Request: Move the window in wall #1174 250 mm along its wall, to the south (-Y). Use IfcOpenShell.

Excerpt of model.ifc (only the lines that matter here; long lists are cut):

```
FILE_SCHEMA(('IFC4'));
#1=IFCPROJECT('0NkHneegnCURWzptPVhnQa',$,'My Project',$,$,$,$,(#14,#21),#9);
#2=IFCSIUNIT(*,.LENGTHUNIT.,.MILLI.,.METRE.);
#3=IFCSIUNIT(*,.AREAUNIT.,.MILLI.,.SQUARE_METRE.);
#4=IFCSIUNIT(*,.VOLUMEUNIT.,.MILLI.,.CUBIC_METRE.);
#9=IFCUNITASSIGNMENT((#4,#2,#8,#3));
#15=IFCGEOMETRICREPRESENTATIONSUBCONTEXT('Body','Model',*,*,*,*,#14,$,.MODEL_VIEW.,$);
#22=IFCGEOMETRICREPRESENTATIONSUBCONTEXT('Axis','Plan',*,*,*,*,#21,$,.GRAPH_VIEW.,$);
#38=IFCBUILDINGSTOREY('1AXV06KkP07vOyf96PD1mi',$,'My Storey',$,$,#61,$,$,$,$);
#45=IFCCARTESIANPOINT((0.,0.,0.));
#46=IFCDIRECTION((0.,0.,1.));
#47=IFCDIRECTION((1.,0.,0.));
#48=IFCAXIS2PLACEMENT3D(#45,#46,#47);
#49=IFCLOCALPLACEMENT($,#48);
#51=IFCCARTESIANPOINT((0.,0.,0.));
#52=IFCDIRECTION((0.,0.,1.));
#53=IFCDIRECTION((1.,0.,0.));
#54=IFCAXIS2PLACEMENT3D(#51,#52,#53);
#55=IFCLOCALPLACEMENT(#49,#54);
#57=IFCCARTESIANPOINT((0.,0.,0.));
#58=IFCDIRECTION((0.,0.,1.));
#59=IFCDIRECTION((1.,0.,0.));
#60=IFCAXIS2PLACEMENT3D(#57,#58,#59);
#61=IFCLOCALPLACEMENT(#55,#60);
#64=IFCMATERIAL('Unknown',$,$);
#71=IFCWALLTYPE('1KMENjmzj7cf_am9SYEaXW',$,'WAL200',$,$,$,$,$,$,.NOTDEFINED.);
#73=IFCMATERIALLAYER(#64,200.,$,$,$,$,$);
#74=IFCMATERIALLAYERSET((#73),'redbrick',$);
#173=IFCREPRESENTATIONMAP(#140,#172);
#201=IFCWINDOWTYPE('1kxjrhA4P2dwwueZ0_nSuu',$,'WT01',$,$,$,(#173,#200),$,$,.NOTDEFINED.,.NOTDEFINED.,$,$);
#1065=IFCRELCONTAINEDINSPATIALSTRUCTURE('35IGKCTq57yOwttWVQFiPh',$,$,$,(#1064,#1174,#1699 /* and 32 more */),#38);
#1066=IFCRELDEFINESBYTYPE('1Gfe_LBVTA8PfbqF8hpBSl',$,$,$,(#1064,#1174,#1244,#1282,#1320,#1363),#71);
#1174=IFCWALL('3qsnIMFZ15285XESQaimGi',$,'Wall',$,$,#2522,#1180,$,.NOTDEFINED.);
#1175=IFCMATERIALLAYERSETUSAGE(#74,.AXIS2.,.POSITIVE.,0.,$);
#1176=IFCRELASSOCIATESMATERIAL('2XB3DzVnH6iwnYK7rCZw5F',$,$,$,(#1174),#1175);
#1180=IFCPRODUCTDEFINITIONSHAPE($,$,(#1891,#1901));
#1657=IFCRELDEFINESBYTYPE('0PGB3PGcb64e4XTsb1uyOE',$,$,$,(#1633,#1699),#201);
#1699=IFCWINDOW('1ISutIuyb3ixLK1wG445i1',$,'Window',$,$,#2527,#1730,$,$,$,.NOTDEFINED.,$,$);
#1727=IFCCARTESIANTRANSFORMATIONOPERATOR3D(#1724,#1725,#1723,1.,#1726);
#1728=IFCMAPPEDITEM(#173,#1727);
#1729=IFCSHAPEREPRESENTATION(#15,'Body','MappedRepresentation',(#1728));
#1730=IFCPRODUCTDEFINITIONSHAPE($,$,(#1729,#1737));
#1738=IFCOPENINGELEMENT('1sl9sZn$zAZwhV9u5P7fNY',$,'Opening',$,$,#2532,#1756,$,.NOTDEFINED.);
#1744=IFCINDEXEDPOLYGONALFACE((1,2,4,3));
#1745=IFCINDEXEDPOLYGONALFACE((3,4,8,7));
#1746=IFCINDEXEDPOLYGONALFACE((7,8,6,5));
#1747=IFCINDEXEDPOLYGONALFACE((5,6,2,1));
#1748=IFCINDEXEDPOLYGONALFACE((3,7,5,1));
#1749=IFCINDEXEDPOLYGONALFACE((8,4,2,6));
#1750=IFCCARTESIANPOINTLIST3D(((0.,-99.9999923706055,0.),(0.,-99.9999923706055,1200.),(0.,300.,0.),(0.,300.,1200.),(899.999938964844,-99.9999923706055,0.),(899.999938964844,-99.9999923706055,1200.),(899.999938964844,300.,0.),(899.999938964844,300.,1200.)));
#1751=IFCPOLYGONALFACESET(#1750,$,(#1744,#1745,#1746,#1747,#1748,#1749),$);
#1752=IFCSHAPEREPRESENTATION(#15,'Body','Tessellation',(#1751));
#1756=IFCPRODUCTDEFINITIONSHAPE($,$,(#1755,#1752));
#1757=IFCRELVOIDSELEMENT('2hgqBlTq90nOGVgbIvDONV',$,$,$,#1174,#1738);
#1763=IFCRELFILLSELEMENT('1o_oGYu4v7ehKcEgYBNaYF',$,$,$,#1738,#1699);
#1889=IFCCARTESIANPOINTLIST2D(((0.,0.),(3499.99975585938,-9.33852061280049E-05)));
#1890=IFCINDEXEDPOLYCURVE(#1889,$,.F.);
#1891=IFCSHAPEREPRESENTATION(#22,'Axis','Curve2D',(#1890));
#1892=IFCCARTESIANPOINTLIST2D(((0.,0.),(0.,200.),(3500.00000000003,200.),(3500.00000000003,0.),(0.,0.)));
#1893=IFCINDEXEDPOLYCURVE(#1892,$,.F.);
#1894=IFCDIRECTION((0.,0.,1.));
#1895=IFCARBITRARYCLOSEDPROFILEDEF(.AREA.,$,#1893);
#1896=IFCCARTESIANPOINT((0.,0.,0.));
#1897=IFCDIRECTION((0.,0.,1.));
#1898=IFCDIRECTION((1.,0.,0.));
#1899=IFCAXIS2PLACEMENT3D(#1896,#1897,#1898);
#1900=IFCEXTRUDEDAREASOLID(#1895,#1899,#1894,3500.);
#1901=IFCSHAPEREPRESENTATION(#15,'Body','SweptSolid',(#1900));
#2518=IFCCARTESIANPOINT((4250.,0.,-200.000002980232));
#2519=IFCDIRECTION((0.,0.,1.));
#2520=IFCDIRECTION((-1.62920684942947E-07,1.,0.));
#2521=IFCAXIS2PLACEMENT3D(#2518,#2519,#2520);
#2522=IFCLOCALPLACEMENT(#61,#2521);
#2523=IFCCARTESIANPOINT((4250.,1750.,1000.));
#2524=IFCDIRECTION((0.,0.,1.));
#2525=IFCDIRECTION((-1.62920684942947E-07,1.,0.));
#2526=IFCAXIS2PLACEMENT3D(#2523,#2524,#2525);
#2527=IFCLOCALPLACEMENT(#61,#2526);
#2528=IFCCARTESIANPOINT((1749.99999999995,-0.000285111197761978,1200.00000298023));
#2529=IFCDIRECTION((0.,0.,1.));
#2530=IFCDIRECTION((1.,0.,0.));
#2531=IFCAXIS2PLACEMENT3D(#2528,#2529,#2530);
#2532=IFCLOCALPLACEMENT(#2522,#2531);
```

```python
import ifcopenshell
import ifcopenshell.api.geometry
import ifcopenshell.util.placement
import ifcopenshell.util.unit

model = ifcopenshell.open("model.ifc")
unit_scale = ifcopenshell.util.unit.calculate_unit_scale(model)

window = model.by_guid("1ISutIuyb3ixLK1wG445i1")
opening = window.FillsVoids[0].RelatingOpeningElement
wall = opening.VoidsElements[0].RelatingBuildingElement

wall_matrix = ifcopenshell.util.placement.get_local_placement(wall.ObjectPlacement)
shift = wall_matrix[:3, 0] * -0.25 / unit_scale
before = ifcopenshell.util.placement.get_local_placement(window.ObjectPlacement)[:3, 3].copy()

# The window is not placed relative to its opening, so move both.
for product in (opening, window):
    matrix = ifcopenshell.util.placement.get_local_placement(product.ObjectPlacement)
    matrix[:3, 3] += shift
    ifcopenshell.api.geometry.edit_object_placement(model, product=product, matrix=matrix, is_si=False)

after = ifcopenshell.util.placement.get_local_placement(window.ObjectPlacement)[:3, 3]
print("window moved by", (after - before).round(3) + 0.0)

model.write("model-out.ifc")
```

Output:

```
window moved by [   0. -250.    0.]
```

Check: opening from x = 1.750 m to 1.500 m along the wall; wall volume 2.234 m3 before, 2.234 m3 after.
